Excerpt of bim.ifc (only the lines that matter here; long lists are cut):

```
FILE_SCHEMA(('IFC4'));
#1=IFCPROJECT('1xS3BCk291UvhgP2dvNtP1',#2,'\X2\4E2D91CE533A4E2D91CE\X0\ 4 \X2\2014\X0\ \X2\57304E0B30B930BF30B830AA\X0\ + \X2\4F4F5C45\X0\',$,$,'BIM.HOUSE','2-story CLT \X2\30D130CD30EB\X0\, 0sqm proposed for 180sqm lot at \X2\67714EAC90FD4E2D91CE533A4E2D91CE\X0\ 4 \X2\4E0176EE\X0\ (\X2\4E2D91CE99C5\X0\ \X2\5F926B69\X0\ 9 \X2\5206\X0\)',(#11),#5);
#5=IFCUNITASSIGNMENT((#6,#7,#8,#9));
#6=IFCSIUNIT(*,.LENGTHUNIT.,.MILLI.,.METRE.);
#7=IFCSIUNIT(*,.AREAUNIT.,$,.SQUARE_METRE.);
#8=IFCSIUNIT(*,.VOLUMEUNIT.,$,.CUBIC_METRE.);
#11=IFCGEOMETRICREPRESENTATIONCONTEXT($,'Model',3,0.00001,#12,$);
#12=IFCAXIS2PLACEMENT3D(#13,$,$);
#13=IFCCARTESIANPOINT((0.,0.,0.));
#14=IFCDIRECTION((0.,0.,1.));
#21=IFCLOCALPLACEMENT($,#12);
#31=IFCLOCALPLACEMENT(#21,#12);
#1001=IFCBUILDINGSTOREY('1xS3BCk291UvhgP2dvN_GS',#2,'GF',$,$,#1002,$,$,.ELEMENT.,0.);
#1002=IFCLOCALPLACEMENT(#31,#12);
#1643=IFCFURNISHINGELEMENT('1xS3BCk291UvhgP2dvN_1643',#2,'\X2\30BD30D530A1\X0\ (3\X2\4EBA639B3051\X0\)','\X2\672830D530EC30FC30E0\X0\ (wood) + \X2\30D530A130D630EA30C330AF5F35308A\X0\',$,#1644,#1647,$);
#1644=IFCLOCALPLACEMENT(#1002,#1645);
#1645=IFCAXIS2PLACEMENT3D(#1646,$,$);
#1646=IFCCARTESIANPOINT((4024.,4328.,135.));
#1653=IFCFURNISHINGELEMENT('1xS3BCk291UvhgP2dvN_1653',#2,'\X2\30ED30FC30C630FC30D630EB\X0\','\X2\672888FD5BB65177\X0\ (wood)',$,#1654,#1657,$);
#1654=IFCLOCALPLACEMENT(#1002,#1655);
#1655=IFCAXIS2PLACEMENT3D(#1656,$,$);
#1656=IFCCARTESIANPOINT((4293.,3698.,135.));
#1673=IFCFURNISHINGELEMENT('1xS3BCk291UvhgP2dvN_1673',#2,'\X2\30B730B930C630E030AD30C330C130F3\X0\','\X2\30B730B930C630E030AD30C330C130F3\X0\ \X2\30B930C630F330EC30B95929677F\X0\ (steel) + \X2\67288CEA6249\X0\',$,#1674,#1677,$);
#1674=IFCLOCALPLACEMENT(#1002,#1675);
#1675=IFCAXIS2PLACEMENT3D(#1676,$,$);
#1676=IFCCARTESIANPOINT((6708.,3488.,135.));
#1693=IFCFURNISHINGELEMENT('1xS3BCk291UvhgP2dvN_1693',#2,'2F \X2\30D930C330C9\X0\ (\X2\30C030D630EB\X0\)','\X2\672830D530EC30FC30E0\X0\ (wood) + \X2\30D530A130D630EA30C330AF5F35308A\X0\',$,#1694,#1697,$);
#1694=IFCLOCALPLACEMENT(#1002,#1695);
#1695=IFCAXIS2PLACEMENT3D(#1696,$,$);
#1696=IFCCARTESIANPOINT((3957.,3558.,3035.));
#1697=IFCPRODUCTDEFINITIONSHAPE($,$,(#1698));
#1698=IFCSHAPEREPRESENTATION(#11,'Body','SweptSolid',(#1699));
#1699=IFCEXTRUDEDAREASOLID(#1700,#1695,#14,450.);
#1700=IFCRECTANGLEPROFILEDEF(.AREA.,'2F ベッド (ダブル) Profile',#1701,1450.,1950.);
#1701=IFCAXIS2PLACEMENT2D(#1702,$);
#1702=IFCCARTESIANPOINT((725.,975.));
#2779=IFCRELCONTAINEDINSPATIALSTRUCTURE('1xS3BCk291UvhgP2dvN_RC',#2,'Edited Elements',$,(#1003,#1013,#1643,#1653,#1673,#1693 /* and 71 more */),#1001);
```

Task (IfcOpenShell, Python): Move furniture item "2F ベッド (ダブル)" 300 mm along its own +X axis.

```python
import ifcopenshell
import ifcopenshell.api.geometry
import ifcopenshell.util.placement

model = ifcopenshell.open("bim.ifc")

item = model.by_guid("1xS3BCk291UvhgP2dvN_1693")
matrix = ifcopenshell.util.placement.get_local_placement(item.ObjectPlacement)
matrix[:3, 3] += matrix[:3, 0] * 300.0
ifcopenshell.api.geometry.edit_object_placement(model, product=item, matrix=matrix, is_si=False)

print(ifcopenshell.util.placement.get_local_placement(item.ObjectPlacement).round(3) + 0.0)

model.write("bim_updated.ifc")
```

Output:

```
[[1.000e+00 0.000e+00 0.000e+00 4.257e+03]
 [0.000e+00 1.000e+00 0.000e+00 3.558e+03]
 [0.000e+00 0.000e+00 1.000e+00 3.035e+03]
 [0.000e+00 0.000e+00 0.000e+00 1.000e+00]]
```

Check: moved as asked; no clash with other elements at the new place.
